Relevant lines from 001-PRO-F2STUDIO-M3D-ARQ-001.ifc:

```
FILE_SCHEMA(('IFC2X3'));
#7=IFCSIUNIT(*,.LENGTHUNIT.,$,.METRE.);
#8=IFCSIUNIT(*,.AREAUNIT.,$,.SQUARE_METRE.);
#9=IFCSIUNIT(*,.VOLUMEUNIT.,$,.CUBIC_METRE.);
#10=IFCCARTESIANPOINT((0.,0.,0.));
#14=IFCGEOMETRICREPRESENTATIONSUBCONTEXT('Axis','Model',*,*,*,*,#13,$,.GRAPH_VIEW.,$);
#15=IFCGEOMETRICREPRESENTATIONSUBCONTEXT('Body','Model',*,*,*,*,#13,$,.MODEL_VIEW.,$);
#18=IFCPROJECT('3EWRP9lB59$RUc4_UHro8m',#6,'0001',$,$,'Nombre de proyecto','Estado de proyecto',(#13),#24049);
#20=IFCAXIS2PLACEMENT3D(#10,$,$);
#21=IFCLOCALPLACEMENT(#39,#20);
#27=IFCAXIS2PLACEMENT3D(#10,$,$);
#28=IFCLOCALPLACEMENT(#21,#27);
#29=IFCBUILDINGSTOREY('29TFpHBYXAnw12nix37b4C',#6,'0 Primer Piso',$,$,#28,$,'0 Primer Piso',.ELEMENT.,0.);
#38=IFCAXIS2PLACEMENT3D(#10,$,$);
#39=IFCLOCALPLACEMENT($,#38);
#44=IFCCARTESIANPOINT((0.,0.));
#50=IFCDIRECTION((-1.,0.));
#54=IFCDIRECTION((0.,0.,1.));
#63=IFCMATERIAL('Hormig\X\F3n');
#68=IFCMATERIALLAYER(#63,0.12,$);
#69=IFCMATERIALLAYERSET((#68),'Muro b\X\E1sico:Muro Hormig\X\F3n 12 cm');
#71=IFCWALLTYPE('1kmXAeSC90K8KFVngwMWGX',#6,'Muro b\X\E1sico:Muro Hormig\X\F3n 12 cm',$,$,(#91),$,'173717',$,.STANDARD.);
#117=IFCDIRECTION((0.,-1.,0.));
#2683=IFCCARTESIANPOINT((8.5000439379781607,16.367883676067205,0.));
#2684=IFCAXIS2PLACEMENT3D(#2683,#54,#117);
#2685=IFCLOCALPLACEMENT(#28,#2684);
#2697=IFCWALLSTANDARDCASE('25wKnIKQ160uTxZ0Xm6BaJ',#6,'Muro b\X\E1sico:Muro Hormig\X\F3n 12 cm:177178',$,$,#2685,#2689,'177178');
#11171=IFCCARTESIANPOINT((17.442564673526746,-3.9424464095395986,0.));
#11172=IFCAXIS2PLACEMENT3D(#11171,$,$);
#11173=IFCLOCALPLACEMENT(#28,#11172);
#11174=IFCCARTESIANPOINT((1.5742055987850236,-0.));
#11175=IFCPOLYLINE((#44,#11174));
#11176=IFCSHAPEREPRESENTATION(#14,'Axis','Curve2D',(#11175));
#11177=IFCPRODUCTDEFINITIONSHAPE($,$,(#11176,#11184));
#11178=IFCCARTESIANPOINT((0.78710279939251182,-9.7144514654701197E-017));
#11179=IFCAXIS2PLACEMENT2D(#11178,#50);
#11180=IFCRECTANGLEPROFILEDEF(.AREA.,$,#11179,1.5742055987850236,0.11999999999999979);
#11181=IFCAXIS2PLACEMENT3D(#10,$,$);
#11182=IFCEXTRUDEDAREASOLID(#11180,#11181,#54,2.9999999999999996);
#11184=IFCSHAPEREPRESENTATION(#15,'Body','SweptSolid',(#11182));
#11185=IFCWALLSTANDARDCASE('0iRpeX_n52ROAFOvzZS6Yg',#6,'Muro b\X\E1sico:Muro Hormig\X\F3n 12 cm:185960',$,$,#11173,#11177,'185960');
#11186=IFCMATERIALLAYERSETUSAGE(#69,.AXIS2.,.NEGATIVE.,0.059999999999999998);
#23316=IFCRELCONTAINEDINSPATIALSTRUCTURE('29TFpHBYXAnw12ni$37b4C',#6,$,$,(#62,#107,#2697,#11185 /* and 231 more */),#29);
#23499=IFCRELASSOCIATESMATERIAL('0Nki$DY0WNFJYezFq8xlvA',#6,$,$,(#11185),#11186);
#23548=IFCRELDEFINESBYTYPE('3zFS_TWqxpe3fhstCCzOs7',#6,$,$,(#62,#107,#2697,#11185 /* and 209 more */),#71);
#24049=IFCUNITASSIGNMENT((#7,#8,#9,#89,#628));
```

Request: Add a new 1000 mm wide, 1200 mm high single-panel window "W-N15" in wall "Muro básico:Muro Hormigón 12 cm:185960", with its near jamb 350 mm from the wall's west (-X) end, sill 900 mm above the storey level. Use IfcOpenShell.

```python
import numpy as np
import ifcopenshell
import ifcopenshell.api.feature
import ifcopenshell.api.geometry
import ifcopenshell.api.root
import ifcopenshell.api.spatial
import ifcopenshell.api.type
import ifcopenshell.geom
import ifcopenshell.util.element
import ifcopenshell.util.placement
import ifcopenshell.util.representation
import ifcopenshell.util.shape
import ifcopenshell.util.unit

model = ifcopenshell.open("001-PRO-F2STUDIO-M3D-ARQ-001.ifc")
unit_scale = ifcopenshell.util.unit.calculate_unit_scale(model)
settings = ifcopenshell.geom.settings()


def volume(element):
    """Net volume in cubic metres, openings subtracted."""
    shape = ifcopenshell.geom.create_shape(settings, element)
    return ifcopenshell.util.shape.get_volume(shape.geometry)


wall = model.by_guid("0iRpeX_n52ROAFOvzZS6Yg")
storey = ifcopenshell.util.element.get_container(wall, ifc_class="IfcBuildingStorey")
context = ifcopenshell.util.representation.get_context(model, "Model", "Body", "MODEL_VIEW")
before = volume(wall)

width, height, from_end, sill = 1, 1.2, 0.35, 0.9  # metres

# The wall runs along its own X axis, and the end named is its -X end.
wall_shape = ifcopenshell.geom.create_shape(settings, wall)
x, y, z = ifcopenshell.util.shape.get_vertices(wall_shape.geometry).T
start = x.min() + from_end
face, thickness = float(y.min()), float(y.max() - y.min())
wall_matrix = ifcopenshell.util.placement.get_local_placement(wall.ObjectPlacement)
level = ifcopenshell.util.placement.get_local_placement(storey.ObjectPlacement)[2, 3]


def in_wall(x, y):
    """Placement at x, y metres in the wall's axes, at sill height."""
    matrix = wall_matrix.copy()
    matrix[:, 3] = wall_matrix @ np.array([x / unit_scale, y / unit_scale, 0.0, 1.0])
    matrix[2, 3] = level + sill / unit_scale
    return matrix


# Opening: a box that overshoots both wall faces by 50 mm.
opening = ifcopenshell.api.root.create_entity(model, ifc_class="IfcOpeningElement")
box = ifcopenshell.api.geometry.add_wall_representation(
    model, context=context, length=width, height=height, thickness=thickness + 0.1
)
ifcopenshell.api.geometry.assign_representation(model, product=opening, representation=box)
ifcopenshell.api.geometry.edit_object_placement(model, product=opening, matrix=in_wall(start, face - 0.05), is_si=False)
ifcopenshell.api.feature.add_feature(model, feature=opening, element=wall)

window = ifcopenshell.api.root.create_entity(model, ifc_class="IfcWindow", name="W-N15")
window.OverallWidth, window.OverallHeight = width / unit_scale, height / unit_scale
body = ifcopenshell.api.geometry.add_window_representation(
    model,
    context=context,
    overall_width=window.OverallWidth,
    overall_height=window.OverallHeight,
    partition_type="SINGLE_PANEL",
)
ifcopenshell.api.geometry.assign_representation(model, product=window, representation=body)
ifcopenshell.api.spatial.assign_container(model, products=[window], relating_structure=storey)
fills = ifcopenshell.api.feature.add_filling(model, opening=opening, element=window)
fills.OwnerHistory = window.OwnerHistory  # required in IFC2X3

# IFC2X3 keeps the operation on the window style.
style = ifcopenshell.api.root.create_entity(model, ifc_class="IfcWindowStyle", name="W-N15")
style.OperationType, style.ConstructionType = "SINGLE_PANEL", "NOTDEFINED"
style.ParameterTakesPrecedence = style.Sizeable = False
ifcopenshell.api.type.assign_type(model, related_objects=[window], relating_type=style)

# Centre the window in the wall's thickness.
ifcopenshell.api.geometry.edit_object_placement(model, product=window, matrix=in_wall(start, face), is_si=False)
window_shape = ifcopenshell.geom.create_shape(settings, window)
depth = ifcopenshell.util.shape.get_vertices(window_shape.geometry)[:, 1]
offset = face + thickness / 2 - (depth.min() + depth.max()) / 2
ifcopenshell.api.geometry.edit_object_placement(model, product=window, matrix=in_wall(start, offset), is_si=False)

after = volume(wall)

print(f"wall volume {before:.3f} -> {after:.3f} m3")

model.write("001-PRO-F2STUDIO-M3D-ARQ-001_edited.ifc")
```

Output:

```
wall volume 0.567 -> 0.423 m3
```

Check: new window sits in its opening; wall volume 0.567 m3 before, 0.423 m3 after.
